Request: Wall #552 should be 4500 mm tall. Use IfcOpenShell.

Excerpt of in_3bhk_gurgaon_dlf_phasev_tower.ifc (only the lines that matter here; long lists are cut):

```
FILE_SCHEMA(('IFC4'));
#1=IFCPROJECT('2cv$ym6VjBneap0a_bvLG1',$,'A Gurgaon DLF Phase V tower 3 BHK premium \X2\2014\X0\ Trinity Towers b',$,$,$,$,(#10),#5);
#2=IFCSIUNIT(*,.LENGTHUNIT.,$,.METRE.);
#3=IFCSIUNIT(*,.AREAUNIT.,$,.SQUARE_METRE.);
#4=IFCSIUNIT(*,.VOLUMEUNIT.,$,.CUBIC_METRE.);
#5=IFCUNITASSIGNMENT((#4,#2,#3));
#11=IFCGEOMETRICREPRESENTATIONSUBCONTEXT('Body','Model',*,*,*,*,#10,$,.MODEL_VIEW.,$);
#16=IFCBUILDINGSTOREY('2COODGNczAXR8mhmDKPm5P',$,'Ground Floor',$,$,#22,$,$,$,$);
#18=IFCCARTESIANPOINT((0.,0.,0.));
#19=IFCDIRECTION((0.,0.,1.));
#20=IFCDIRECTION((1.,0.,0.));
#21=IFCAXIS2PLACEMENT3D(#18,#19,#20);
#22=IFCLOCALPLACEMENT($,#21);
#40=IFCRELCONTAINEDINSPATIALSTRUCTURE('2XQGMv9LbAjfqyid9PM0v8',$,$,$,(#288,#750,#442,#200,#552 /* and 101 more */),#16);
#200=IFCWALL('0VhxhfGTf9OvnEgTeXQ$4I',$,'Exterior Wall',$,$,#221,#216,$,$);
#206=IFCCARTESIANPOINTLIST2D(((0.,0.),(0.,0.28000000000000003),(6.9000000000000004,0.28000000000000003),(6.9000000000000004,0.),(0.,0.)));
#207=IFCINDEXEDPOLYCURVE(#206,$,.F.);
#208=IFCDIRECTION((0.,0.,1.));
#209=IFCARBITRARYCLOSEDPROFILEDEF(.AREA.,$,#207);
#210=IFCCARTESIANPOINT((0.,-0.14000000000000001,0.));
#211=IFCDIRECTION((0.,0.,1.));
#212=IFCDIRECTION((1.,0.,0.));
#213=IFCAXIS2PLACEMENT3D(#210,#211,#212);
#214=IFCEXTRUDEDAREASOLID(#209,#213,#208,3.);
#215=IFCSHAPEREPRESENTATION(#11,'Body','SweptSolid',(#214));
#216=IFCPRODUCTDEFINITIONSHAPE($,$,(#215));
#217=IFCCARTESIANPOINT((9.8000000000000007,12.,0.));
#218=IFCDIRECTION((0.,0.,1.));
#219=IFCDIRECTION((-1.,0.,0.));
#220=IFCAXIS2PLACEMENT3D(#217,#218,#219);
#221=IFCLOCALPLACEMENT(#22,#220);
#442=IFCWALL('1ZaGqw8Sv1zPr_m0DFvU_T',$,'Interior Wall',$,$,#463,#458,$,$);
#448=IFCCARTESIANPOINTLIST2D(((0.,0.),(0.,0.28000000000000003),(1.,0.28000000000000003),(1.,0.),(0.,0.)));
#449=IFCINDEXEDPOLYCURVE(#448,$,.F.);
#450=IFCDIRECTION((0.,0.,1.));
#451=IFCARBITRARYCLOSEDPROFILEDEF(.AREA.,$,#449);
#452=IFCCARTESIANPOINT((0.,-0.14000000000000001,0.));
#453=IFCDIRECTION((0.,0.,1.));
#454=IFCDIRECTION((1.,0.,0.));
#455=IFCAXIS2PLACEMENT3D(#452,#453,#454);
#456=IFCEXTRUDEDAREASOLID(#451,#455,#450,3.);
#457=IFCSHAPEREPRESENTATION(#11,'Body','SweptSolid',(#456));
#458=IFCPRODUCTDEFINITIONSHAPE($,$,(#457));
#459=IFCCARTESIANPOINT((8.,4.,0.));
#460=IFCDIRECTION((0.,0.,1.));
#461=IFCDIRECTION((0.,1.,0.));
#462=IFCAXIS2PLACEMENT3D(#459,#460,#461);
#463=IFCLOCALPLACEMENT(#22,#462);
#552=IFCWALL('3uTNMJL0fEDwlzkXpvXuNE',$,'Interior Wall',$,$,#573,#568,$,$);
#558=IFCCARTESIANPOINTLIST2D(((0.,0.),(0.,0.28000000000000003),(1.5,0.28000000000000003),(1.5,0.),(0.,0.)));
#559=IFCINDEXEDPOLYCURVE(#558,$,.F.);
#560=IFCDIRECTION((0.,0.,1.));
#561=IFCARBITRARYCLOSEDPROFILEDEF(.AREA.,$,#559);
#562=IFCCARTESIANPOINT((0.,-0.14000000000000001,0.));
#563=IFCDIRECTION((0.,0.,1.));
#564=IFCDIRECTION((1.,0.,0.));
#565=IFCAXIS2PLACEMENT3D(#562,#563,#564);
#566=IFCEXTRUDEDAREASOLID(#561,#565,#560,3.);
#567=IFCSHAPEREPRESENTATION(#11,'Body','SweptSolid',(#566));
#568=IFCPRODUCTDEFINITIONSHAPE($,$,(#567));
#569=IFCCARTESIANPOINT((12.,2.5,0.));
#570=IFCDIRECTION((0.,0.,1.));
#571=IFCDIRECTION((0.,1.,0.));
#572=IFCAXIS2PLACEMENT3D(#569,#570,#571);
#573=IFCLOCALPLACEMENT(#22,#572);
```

```python
import ifcopenshell
import ifcopenshell.geom
import ifcopenshell.util.representation
import ifcopenshell.util.shape
import ifcopenshell.util.unit

model = ifcopenshell.open("in_3bhk_gurgaon_dlf_phasev_tower.ifc")
unit_scale = ifcopenshell.util.unit.calculate_unit_scale(model)
settings = ifcopenshell.geom.settings()


def volume(element):
    """Net volume in cubic metres, openings subtracted."""
    shape = ifcopenshell.geom.create_shape(settings, element)
    return ifcopenshell.util.shape.get_volume(shape.geometry)


wall = model.by_guid("3uTNMJL0fEDwlzkXpvXuNE")
before = volume(wall)

body = ifcopenshell.util.representation.get_representation(wall, "Model", "Body")
solid = body.Items[0]
old_height = solid.Depth
solid.Depth = 4.5 / unit_scale
after = volume(wall)

print(f"height {old_height:g} -> {solid.Depth:g}, volume {before:.3f} -> {after:.3f} m3")

model.write("in_3bhk_gurgaon_dlf_phasev_tower-out.ifc")
```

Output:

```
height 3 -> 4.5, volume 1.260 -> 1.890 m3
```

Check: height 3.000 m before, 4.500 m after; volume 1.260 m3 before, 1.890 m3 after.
